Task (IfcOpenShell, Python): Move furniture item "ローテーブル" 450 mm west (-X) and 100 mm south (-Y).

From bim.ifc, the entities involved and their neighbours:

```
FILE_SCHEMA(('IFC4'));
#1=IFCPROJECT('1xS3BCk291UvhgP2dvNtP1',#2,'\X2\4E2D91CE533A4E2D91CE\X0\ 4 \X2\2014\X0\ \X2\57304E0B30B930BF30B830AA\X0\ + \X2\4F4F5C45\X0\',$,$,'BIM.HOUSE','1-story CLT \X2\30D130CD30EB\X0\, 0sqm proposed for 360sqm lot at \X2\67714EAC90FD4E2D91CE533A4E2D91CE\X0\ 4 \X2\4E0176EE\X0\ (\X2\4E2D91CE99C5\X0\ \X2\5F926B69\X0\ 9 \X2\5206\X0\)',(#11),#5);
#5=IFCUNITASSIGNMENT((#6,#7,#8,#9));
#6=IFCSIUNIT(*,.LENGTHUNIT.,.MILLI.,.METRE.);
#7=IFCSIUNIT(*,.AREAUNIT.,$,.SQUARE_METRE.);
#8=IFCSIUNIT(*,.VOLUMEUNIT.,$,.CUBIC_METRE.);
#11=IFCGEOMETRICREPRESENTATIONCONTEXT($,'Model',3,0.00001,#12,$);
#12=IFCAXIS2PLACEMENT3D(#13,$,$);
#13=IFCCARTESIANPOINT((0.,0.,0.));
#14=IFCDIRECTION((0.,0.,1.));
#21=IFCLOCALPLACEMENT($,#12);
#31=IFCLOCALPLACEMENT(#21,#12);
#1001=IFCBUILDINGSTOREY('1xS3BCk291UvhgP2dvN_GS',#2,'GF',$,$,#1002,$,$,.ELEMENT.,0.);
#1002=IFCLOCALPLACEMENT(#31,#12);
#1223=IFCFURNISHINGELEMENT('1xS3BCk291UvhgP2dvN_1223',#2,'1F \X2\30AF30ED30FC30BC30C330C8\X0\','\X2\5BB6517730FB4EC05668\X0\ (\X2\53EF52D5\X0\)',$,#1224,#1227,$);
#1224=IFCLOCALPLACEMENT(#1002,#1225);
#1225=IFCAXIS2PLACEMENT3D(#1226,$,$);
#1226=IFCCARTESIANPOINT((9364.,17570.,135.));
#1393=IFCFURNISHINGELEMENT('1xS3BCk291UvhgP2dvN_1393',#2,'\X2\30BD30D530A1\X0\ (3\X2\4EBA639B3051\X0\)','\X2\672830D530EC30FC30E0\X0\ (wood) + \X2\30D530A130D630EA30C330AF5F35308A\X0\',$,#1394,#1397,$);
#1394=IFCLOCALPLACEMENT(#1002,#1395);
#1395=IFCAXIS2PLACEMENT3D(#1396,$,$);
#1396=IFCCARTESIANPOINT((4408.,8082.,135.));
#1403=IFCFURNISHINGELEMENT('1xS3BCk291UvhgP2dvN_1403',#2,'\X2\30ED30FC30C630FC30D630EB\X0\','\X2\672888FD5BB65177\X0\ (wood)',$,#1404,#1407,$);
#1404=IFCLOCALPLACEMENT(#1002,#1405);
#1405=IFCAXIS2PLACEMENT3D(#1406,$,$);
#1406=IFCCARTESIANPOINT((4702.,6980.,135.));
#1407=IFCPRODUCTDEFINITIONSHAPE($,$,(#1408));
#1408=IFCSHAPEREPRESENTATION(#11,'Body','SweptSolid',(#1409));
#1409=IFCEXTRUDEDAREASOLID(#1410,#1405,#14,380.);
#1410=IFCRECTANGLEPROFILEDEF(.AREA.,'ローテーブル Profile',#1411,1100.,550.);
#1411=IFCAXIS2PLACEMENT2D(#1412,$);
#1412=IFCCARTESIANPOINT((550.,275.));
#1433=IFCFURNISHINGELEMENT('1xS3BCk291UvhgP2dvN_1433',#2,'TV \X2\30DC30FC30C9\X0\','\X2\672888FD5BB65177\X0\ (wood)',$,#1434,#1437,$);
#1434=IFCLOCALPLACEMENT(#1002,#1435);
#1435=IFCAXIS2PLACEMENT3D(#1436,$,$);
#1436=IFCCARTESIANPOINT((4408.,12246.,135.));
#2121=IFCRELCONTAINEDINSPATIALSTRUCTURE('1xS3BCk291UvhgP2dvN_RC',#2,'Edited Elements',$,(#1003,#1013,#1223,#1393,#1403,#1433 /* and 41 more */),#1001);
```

```python
import ifcopenshell
import ifcopenshell.api.geometry
import ifcopenshell.util.placement
import ifcopenshell.util.unit

model = ifcopenshell.open("bim.ifc")
unit_scale = ifcopenshell.util.unit.calculate_unit_scale(model)

item = model.by_guid("1xS3BCk291UvhgP2dvN_1403")
matrix = ifcopenshell.util.placement.get_local_placement(item.ObjectPlacement)
matrix[0, 3] -= 0.45 / unit_scale
matrix[1, 3] -= 0.1 / unit_scale
ifcopenshell.api.geometry.edit_object_placement(model, product=item, matrix=matrix, is_si=False)

print(ifcopenshell.util.placement.get_local_placement(item.ObjectPlacement).round(3) + 0.0)

model.write("bim-out.ifc")
```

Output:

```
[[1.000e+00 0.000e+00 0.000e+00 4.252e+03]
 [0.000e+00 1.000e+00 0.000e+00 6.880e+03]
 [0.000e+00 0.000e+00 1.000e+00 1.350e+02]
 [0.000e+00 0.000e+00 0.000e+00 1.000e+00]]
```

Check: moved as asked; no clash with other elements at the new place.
